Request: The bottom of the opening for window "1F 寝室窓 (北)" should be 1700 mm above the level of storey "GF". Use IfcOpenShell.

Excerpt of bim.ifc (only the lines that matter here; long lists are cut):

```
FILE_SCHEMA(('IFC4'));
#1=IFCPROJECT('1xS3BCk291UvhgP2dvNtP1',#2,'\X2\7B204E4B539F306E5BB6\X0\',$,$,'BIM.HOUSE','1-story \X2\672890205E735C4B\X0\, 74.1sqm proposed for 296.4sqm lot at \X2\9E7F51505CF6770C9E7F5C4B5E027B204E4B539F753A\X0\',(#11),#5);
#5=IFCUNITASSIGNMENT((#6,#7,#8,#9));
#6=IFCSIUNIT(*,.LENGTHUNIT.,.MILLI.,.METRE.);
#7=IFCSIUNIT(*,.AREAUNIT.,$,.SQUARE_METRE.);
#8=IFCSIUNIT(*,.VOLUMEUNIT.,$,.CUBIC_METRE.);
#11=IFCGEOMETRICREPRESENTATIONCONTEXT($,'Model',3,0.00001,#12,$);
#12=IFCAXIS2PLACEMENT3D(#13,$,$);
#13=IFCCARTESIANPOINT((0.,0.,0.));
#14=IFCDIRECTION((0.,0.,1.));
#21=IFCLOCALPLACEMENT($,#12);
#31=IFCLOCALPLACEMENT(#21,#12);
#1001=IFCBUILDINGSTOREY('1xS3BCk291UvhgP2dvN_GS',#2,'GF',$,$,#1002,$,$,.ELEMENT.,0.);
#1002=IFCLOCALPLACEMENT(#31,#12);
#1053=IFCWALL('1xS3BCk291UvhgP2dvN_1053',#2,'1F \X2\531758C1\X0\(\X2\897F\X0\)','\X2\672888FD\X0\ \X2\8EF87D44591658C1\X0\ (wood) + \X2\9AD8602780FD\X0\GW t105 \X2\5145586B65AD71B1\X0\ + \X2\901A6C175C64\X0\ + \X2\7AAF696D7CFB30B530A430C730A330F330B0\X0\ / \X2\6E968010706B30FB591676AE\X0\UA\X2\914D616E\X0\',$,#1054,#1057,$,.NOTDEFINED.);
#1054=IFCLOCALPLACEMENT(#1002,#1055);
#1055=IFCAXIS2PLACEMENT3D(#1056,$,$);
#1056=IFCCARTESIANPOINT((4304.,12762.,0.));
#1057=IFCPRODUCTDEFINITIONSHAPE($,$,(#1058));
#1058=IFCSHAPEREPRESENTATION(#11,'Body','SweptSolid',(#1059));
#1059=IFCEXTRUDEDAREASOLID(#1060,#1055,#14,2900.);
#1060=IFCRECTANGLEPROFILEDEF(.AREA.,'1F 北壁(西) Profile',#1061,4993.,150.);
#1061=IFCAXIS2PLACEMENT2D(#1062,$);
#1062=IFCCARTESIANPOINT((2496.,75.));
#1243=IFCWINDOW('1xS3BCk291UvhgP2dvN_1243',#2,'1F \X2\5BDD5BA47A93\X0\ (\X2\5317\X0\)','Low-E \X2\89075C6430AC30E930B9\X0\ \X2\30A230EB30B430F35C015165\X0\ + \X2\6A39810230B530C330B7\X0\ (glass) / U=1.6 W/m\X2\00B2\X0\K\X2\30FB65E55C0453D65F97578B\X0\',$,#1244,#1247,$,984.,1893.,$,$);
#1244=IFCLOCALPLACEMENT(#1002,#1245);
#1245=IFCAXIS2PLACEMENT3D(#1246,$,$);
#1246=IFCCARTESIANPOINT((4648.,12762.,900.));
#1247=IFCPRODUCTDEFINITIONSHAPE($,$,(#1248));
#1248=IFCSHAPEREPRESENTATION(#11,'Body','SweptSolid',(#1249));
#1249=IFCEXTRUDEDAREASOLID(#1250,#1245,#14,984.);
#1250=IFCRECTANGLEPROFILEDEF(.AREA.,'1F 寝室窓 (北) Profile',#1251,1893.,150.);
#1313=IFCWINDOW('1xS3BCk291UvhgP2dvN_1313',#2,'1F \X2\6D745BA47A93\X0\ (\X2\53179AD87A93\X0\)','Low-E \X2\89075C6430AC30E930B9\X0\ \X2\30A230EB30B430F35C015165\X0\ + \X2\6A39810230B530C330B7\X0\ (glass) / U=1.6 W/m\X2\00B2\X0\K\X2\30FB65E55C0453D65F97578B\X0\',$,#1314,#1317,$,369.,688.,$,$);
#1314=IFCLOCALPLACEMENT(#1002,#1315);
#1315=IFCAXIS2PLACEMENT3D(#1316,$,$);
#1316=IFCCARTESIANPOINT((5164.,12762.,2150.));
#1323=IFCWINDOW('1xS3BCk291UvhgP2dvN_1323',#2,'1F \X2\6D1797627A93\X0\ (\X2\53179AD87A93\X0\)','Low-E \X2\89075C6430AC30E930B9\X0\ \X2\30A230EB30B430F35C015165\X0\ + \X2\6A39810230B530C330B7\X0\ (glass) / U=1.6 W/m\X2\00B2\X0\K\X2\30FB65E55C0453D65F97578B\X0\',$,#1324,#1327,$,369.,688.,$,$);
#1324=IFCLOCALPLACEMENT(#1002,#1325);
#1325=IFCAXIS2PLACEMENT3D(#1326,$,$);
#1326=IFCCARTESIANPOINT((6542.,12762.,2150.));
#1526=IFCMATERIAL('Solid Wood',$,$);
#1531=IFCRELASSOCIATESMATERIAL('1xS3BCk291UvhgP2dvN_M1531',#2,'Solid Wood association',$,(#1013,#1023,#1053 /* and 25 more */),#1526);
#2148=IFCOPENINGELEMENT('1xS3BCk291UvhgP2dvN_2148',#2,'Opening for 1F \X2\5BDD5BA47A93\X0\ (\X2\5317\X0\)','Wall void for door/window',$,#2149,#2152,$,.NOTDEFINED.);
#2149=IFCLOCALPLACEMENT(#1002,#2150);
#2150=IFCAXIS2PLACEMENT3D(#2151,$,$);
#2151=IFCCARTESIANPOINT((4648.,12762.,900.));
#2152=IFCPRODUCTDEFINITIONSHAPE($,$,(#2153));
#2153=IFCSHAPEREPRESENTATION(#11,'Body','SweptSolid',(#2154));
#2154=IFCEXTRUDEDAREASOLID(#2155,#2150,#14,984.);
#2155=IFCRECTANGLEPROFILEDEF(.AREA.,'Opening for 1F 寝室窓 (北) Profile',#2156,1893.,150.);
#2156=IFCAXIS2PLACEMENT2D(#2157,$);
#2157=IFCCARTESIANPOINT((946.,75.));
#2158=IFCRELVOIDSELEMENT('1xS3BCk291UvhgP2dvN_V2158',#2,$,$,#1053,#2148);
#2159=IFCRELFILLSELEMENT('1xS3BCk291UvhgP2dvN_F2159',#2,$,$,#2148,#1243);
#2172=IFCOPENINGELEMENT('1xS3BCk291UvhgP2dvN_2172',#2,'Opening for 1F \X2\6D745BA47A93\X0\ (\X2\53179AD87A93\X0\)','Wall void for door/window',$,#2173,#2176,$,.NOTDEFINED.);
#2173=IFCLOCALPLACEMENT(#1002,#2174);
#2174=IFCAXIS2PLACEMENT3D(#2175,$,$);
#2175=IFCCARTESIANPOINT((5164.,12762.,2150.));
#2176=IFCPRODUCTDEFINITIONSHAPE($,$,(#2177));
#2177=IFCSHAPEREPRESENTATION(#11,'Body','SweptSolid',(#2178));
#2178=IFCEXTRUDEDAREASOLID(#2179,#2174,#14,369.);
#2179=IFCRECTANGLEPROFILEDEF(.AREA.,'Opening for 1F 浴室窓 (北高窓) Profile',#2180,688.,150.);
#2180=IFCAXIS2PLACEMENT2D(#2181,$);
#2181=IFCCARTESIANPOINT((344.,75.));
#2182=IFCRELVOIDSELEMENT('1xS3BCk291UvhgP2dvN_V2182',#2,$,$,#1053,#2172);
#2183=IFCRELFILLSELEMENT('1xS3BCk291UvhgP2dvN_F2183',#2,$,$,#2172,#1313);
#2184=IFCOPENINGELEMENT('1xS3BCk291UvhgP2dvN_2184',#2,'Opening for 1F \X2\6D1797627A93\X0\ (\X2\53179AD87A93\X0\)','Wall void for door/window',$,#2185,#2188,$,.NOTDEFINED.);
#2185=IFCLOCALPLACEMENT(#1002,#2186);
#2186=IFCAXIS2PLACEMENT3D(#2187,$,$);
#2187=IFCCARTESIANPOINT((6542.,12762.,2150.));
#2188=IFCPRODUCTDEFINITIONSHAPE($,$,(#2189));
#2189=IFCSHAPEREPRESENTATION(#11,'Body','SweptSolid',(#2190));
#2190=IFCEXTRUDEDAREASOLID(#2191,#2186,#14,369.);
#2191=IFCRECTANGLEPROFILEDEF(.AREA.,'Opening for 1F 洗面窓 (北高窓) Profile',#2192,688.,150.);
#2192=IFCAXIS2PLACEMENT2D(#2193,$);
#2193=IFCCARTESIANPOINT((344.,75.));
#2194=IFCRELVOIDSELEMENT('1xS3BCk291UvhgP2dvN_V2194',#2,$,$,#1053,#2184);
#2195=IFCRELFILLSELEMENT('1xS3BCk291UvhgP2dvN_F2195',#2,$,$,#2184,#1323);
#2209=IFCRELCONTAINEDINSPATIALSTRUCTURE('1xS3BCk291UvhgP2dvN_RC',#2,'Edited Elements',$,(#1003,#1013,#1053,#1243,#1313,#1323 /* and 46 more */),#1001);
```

```python
import numpy as np
import ifcopenshell
import ifcopenshell.api.geometry
import ifcopenshell.geom
import ifcopenshell.util.element
import ifcopenshell.util.placement
import ifcopenshell.util.shape
import ifcopenshell.util.unit

model = ifcopenshell.open("bim.ifc")
unit_scale = ifcopenshell.util.unit.calculate_unit_scale(model)

window = model.by_guid("1xS3BCk291UvhgP2dvN_1243")
opening = window.FillsVoids[0].RelatingOpeningElement
storey = ifcopenshell.util.element.get_container(window, ifc_class="IfcBuildingStorey")
level = ifcopenshell.util.placement.get_local_placement(storey.ObjectPlacement)[2, 3]

# The opening's origin need not be at the sill, so measure its lowest point.
shape = ifcopenshell.geom.create_shape(ifcopenshell.geom.settings(), opening)
bottom = ifcopenshell.util.shape.get_shape_bottom_elevation(shape, shape.geometry) / unit_scale
dz = level + 1700.0 - bottom

shift = np.array([0.0, 0.0, dz])
# The window is not placed relative to its opening, so move both.
for product in (opening, window):
    matrix = ifcopenshell.util.placement.get_local_placement(product.ObjectPlacement)
    matrix[:3, 3] += shift
    ifcopenshell.api.geometry.edit_object_placement(model, product=product, matrix=matrix, is_si=False)

print(f"moved by {dz * unit_scale:+.3f} m")

model.write("bim_rev.ifc")
```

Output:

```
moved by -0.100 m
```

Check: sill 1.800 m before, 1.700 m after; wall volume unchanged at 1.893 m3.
